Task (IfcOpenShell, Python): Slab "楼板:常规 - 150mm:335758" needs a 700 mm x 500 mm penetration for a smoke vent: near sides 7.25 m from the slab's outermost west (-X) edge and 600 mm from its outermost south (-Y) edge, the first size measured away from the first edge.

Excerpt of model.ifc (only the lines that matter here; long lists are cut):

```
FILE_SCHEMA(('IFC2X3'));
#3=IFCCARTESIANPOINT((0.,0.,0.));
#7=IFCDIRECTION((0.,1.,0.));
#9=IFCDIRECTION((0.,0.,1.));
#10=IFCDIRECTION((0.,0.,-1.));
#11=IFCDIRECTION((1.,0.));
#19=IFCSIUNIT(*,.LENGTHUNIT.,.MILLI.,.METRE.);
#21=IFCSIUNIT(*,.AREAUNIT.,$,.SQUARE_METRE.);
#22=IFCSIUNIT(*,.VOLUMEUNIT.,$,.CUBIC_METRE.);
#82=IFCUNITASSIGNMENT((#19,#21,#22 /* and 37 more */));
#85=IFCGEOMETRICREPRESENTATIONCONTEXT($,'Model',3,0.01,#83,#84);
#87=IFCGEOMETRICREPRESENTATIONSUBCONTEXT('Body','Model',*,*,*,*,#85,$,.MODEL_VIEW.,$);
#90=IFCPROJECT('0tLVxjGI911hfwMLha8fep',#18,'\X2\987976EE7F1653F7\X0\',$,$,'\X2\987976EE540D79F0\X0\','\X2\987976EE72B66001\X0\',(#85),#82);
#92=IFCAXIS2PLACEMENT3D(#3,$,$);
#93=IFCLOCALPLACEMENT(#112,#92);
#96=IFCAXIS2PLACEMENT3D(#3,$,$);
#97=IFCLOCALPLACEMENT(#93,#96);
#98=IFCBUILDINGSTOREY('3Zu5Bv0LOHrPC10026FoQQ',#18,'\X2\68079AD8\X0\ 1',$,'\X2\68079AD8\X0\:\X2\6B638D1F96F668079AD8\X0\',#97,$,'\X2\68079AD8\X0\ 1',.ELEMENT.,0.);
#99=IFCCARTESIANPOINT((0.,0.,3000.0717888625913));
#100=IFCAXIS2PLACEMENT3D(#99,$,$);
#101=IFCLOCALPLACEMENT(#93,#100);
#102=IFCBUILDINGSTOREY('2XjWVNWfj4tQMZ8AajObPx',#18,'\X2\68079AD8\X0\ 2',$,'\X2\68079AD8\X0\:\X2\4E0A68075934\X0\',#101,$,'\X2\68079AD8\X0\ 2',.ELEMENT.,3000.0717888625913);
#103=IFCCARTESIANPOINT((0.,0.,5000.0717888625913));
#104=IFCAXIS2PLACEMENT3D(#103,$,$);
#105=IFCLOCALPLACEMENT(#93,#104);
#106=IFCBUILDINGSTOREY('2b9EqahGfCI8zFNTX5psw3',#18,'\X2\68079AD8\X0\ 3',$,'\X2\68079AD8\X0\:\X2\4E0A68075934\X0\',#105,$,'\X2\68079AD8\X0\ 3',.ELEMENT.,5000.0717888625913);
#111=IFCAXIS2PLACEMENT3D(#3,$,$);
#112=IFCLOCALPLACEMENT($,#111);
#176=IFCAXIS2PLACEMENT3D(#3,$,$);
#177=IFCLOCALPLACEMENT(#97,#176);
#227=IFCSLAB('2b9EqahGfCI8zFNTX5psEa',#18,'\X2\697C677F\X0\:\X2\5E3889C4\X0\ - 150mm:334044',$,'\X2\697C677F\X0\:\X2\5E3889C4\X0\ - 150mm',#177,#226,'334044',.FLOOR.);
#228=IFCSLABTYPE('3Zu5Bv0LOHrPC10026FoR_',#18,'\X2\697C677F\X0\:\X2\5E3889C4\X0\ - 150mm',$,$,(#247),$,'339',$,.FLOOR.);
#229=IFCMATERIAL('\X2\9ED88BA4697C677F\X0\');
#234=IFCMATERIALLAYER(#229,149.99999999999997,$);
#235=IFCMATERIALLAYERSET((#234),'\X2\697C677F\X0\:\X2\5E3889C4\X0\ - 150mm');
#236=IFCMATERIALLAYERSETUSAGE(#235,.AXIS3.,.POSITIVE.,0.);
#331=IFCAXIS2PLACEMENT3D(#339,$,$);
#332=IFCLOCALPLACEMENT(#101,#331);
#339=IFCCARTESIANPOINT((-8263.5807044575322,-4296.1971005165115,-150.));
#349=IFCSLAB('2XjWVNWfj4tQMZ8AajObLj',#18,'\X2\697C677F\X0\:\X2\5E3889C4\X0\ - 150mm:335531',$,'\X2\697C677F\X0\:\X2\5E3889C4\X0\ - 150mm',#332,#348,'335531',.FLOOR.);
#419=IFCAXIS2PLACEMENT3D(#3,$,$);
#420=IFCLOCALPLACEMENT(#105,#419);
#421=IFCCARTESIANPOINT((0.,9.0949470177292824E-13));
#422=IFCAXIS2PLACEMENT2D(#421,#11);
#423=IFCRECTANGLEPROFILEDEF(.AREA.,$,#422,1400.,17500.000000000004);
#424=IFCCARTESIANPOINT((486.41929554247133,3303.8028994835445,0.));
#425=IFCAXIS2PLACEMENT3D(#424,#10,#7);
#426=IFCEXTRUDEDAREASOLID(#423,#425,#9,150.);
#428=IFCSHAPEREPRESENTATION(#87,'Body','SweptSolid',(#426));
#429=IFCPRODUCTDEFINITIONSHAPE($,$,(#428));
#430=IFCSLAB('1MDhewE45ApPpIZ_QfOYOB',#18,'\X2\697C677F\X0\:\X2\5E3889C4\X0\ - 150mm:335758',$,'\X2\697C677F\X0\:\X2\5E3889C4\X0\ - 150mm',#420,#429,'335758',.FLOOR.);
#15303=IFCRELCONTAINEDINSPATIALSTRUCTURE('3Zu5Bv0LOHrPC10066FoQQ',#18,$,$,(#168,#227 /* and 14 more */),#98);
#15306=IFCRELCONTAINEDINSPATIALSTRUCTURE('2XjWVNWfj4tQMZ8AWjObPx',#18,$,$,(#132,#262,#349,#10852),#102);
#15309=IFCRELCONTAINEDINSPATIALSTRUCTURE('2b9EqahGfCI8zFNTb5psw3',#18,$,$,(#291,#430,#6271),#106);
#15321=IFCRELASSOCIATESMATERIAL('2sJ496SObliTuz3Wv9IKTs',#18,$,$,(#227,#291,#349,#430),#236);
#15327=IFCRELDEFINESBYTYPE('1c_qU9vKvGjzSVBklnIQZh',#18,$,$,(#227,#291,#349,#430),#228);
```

```python
import numpy as np
import ifcopenshell
import ifcopenshell.api.feature
import ifcopenshell.api.geometry
import ifcopenshell.api.root
import ifcopenshell.geom
import ifcopenshell.util.placement
import ifcopenshell.util.representation
import ifcopenshell.util.shape
import ifcopenshell.util.unit

model = ifcopenshell.open("model.ifc")
unit_scale = ifcopenshell.util.unit.calculate_unit_scale(model)
settings = ifcopenshell.geom.settings()


def volume(element):
    """Net volume in cubic metres, openings subtracted."""
    shape = ifcopenshell.geom.create_shape(settings, element)
    return ifcopenshell.util.shape.get_volume(shape.geometry)


slab = model.by_guid("1MDhewE45ApPpIZ_QfOYOB")
before = volume(slab)

# Extent in the slab's own axes, in metres. The edges named are its -X and -Y sides.
slab_shape = ifcopenshell.geom.create_shape(settings, slab)
vertices = ifcopenshell.util.shape.get_vertices(slab_shape.geometry)
x_min, y_min, bottom = vertices.min(axis=0)
top = vertices[:, 2].max()

opening = ifcopenshell.api.root.create_entity(model, ifc_class="IfcOpeningElement", name="Smoke vent opening")
context = ifcopenshell.util.representation.get_context(model, "Model", "Body", "MODEL_VIEW")
width, depth = 0.7, 0.5
outline = [(0.0, 0.0), (width, 0.0), (width, depth), (0.0, depth), (0.0, 0.0)]
# Overshoot both faces by 50 mm so the cut is clean.
shape = ifcopenshell.api.geometry.add_slab_representation(
    model, context=context, depth=top - bottom + 0.1, polyline=outline
)
ifcopenshell.api.geometry.assign_representation(model, product=opening, representation=shape)

matrix = ifcopenshell.util.placement.get_local_placement(slab.ObjectPlacement)
matrix[:, 3] = matrix @ np.append(np.array([x_min + 7.25, y_min + 0.6, bottom - 0.05]) / unit_scale, 1.0)
ifcopenshell.api.geometry.edit_object_placement(model, product=opening, matrix=matrix, is_si=False)
ifcopenshell.api.feature.add_feature(model, feature=opening, element=slab)

after = volume(slab)

print(f"slab volume {before:.3f} -> {after:.3f} m3")

model.write("model_edited.ifc")
```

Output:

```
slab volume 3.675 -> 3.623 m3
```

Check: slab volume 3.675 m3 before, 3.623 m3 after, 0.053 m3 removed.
